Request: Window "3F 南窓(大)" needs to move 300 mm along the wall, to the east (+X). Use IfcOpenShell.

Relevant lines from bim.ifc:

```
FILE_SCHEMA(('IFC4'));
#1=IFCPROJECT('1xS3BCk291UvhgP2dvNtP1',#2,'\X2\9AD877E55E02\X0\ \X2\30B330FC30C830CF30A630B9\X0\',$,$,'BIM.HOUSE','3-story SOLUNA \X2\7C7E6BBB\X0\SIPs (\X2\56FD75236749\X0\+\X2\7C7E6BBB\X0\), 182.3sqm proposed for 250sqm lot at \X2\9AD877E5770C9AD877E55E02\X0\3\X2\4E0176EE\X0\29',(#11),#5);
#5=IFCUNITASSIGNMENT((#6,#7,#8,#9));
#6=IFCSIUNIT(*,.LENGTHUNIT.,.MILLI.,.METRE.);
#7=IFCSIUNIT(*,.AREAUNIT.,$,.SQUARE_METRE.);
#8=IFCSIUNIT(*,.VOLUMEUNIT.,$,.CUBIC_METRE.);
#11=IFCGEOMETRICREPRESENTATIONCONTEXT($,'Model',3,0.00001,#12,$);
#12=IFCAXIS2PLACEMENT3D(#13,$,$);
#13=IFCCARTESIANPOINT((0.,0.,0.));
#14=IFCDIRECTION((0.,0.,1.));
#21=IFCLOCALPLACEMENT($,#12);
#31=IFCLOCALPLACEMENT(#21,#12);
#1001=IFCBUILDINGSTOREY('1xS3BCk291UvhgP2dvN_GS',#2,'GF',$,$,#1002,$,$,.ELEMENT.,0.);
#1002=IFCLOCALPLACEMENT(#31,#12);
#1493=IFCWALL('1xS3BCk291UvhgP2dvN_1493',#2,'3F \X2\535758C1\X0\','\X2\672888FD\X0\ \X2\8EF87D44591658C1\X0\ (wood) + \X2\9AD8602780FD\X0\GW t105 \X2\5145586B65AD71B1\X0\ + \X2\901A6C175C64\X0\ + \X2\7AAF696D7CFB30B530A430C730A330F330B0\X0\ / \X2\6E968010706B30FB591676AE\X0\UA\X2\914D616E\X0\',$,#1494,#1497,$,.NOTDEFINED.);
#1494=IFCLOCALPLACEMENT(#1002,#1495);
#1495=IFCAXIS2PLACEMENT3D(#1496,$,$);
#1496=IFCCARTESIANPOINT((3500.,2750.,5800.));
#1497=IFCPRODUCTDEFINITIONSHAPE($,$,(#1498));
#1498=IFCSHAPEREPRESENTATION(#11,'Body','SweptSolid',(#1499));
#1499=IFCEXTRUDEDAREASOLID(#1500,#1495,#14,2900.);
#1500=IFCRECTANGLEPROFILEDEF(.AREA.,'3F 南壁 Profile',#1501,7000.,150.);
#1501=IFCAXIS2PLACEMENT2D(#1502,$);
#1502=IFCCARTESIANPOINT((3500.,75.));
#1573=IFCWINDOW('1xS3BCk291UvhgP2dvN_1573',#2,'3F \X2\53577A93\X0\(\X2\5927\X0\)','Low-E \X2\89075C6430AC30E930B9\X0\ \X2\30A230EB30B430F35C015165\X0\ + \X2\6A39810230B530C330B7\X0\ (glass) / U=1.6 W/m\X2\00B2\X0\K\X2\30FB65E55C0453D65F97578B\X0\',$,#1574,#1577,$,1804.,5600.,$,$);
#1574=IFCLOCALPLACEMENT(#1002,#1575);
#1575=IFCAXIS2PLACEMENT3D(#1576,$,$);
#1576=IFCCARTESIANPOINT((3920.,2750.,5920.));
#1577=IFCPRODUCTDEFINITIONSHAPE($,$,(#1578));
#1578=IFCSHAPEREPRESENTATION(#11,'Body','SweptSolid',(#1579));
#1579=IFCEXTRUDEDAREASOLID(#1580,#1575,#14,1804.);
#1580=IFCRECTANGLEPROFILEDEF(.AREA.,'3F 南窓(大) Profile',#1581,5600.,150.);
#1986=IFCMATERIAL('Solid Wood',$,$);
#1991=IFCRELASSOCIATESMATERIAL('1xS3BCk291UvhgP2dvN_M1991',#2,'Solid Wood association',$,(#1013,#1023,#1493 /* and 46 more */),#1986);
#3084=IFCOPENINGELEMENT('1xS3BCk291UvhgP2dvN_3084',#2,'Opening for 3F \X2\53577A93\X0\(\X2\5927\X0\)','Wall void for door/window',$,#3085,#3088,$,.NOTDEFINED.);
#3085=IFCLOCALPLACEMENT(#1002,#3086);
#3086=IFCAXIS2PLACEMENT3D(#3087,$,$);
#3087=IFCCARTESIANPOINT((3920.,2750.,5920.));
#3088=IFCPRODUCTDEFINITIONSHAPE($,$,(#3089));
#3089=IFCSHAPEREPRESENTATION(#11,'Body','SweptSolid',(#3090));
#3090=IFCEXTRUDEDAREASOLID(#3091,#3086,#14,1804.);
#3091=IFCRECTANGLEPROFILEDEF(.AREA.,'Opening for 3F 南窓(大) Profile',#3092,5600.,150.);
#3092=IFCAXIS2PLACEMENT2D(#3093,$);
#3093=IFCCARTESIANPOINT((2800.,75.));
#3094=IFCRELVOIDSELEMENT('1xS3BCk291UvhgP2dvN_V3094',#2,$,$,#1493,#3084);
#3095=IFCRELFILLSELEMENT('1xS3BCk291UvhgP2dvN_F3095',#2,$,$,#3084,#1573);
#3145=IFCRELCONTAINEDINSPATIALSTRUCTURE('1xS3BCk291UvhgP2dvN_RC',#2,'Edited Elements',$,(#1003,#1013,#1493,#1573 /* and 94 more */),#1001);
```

```python
import ifcopenshell
import ifcopenshell.api.geometry
import ifcopenshell.util.placement

model = ifcopenshell.open("bim.ifc")

window = model.by_id(1573)
opening = window.FillsVoids[0].RelatingOpeningElement
wall = opening.VoidsElements[0].RelatingBuildingElement

wall_matrix = ifcopenshell.util.placement.get_local_placement(wall.ObjectPlacement)
shift = wall_matrix[:3, 0] * 300.0
before = ifcopenshell.util.placement.get_local_placement(window.ObjectPlacement)[:3, 3].copy()

# The window is not placed relative to its opening, so move both.
for product in (opening, window):
    matrix = ifcopenshell.util.placement.get_local_placement(product.ObjectPlacement)
    matrix[:3, 3] += shift
    ifcopenshell.api.geometry.edit_object_placement(model, product=product, matrix=matrix, is_si=False)

after = ifcopenshell.util.placement.get_local_placement(window.ObjectPlacement)[:3, 3]
print("window moved by", (after - before).round(3) + 0.0)

model.write("bim_v2.ifc")
```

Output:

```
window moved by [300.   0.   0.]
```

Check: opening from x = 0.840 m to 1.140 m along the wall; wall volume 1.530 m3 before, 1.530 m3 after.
